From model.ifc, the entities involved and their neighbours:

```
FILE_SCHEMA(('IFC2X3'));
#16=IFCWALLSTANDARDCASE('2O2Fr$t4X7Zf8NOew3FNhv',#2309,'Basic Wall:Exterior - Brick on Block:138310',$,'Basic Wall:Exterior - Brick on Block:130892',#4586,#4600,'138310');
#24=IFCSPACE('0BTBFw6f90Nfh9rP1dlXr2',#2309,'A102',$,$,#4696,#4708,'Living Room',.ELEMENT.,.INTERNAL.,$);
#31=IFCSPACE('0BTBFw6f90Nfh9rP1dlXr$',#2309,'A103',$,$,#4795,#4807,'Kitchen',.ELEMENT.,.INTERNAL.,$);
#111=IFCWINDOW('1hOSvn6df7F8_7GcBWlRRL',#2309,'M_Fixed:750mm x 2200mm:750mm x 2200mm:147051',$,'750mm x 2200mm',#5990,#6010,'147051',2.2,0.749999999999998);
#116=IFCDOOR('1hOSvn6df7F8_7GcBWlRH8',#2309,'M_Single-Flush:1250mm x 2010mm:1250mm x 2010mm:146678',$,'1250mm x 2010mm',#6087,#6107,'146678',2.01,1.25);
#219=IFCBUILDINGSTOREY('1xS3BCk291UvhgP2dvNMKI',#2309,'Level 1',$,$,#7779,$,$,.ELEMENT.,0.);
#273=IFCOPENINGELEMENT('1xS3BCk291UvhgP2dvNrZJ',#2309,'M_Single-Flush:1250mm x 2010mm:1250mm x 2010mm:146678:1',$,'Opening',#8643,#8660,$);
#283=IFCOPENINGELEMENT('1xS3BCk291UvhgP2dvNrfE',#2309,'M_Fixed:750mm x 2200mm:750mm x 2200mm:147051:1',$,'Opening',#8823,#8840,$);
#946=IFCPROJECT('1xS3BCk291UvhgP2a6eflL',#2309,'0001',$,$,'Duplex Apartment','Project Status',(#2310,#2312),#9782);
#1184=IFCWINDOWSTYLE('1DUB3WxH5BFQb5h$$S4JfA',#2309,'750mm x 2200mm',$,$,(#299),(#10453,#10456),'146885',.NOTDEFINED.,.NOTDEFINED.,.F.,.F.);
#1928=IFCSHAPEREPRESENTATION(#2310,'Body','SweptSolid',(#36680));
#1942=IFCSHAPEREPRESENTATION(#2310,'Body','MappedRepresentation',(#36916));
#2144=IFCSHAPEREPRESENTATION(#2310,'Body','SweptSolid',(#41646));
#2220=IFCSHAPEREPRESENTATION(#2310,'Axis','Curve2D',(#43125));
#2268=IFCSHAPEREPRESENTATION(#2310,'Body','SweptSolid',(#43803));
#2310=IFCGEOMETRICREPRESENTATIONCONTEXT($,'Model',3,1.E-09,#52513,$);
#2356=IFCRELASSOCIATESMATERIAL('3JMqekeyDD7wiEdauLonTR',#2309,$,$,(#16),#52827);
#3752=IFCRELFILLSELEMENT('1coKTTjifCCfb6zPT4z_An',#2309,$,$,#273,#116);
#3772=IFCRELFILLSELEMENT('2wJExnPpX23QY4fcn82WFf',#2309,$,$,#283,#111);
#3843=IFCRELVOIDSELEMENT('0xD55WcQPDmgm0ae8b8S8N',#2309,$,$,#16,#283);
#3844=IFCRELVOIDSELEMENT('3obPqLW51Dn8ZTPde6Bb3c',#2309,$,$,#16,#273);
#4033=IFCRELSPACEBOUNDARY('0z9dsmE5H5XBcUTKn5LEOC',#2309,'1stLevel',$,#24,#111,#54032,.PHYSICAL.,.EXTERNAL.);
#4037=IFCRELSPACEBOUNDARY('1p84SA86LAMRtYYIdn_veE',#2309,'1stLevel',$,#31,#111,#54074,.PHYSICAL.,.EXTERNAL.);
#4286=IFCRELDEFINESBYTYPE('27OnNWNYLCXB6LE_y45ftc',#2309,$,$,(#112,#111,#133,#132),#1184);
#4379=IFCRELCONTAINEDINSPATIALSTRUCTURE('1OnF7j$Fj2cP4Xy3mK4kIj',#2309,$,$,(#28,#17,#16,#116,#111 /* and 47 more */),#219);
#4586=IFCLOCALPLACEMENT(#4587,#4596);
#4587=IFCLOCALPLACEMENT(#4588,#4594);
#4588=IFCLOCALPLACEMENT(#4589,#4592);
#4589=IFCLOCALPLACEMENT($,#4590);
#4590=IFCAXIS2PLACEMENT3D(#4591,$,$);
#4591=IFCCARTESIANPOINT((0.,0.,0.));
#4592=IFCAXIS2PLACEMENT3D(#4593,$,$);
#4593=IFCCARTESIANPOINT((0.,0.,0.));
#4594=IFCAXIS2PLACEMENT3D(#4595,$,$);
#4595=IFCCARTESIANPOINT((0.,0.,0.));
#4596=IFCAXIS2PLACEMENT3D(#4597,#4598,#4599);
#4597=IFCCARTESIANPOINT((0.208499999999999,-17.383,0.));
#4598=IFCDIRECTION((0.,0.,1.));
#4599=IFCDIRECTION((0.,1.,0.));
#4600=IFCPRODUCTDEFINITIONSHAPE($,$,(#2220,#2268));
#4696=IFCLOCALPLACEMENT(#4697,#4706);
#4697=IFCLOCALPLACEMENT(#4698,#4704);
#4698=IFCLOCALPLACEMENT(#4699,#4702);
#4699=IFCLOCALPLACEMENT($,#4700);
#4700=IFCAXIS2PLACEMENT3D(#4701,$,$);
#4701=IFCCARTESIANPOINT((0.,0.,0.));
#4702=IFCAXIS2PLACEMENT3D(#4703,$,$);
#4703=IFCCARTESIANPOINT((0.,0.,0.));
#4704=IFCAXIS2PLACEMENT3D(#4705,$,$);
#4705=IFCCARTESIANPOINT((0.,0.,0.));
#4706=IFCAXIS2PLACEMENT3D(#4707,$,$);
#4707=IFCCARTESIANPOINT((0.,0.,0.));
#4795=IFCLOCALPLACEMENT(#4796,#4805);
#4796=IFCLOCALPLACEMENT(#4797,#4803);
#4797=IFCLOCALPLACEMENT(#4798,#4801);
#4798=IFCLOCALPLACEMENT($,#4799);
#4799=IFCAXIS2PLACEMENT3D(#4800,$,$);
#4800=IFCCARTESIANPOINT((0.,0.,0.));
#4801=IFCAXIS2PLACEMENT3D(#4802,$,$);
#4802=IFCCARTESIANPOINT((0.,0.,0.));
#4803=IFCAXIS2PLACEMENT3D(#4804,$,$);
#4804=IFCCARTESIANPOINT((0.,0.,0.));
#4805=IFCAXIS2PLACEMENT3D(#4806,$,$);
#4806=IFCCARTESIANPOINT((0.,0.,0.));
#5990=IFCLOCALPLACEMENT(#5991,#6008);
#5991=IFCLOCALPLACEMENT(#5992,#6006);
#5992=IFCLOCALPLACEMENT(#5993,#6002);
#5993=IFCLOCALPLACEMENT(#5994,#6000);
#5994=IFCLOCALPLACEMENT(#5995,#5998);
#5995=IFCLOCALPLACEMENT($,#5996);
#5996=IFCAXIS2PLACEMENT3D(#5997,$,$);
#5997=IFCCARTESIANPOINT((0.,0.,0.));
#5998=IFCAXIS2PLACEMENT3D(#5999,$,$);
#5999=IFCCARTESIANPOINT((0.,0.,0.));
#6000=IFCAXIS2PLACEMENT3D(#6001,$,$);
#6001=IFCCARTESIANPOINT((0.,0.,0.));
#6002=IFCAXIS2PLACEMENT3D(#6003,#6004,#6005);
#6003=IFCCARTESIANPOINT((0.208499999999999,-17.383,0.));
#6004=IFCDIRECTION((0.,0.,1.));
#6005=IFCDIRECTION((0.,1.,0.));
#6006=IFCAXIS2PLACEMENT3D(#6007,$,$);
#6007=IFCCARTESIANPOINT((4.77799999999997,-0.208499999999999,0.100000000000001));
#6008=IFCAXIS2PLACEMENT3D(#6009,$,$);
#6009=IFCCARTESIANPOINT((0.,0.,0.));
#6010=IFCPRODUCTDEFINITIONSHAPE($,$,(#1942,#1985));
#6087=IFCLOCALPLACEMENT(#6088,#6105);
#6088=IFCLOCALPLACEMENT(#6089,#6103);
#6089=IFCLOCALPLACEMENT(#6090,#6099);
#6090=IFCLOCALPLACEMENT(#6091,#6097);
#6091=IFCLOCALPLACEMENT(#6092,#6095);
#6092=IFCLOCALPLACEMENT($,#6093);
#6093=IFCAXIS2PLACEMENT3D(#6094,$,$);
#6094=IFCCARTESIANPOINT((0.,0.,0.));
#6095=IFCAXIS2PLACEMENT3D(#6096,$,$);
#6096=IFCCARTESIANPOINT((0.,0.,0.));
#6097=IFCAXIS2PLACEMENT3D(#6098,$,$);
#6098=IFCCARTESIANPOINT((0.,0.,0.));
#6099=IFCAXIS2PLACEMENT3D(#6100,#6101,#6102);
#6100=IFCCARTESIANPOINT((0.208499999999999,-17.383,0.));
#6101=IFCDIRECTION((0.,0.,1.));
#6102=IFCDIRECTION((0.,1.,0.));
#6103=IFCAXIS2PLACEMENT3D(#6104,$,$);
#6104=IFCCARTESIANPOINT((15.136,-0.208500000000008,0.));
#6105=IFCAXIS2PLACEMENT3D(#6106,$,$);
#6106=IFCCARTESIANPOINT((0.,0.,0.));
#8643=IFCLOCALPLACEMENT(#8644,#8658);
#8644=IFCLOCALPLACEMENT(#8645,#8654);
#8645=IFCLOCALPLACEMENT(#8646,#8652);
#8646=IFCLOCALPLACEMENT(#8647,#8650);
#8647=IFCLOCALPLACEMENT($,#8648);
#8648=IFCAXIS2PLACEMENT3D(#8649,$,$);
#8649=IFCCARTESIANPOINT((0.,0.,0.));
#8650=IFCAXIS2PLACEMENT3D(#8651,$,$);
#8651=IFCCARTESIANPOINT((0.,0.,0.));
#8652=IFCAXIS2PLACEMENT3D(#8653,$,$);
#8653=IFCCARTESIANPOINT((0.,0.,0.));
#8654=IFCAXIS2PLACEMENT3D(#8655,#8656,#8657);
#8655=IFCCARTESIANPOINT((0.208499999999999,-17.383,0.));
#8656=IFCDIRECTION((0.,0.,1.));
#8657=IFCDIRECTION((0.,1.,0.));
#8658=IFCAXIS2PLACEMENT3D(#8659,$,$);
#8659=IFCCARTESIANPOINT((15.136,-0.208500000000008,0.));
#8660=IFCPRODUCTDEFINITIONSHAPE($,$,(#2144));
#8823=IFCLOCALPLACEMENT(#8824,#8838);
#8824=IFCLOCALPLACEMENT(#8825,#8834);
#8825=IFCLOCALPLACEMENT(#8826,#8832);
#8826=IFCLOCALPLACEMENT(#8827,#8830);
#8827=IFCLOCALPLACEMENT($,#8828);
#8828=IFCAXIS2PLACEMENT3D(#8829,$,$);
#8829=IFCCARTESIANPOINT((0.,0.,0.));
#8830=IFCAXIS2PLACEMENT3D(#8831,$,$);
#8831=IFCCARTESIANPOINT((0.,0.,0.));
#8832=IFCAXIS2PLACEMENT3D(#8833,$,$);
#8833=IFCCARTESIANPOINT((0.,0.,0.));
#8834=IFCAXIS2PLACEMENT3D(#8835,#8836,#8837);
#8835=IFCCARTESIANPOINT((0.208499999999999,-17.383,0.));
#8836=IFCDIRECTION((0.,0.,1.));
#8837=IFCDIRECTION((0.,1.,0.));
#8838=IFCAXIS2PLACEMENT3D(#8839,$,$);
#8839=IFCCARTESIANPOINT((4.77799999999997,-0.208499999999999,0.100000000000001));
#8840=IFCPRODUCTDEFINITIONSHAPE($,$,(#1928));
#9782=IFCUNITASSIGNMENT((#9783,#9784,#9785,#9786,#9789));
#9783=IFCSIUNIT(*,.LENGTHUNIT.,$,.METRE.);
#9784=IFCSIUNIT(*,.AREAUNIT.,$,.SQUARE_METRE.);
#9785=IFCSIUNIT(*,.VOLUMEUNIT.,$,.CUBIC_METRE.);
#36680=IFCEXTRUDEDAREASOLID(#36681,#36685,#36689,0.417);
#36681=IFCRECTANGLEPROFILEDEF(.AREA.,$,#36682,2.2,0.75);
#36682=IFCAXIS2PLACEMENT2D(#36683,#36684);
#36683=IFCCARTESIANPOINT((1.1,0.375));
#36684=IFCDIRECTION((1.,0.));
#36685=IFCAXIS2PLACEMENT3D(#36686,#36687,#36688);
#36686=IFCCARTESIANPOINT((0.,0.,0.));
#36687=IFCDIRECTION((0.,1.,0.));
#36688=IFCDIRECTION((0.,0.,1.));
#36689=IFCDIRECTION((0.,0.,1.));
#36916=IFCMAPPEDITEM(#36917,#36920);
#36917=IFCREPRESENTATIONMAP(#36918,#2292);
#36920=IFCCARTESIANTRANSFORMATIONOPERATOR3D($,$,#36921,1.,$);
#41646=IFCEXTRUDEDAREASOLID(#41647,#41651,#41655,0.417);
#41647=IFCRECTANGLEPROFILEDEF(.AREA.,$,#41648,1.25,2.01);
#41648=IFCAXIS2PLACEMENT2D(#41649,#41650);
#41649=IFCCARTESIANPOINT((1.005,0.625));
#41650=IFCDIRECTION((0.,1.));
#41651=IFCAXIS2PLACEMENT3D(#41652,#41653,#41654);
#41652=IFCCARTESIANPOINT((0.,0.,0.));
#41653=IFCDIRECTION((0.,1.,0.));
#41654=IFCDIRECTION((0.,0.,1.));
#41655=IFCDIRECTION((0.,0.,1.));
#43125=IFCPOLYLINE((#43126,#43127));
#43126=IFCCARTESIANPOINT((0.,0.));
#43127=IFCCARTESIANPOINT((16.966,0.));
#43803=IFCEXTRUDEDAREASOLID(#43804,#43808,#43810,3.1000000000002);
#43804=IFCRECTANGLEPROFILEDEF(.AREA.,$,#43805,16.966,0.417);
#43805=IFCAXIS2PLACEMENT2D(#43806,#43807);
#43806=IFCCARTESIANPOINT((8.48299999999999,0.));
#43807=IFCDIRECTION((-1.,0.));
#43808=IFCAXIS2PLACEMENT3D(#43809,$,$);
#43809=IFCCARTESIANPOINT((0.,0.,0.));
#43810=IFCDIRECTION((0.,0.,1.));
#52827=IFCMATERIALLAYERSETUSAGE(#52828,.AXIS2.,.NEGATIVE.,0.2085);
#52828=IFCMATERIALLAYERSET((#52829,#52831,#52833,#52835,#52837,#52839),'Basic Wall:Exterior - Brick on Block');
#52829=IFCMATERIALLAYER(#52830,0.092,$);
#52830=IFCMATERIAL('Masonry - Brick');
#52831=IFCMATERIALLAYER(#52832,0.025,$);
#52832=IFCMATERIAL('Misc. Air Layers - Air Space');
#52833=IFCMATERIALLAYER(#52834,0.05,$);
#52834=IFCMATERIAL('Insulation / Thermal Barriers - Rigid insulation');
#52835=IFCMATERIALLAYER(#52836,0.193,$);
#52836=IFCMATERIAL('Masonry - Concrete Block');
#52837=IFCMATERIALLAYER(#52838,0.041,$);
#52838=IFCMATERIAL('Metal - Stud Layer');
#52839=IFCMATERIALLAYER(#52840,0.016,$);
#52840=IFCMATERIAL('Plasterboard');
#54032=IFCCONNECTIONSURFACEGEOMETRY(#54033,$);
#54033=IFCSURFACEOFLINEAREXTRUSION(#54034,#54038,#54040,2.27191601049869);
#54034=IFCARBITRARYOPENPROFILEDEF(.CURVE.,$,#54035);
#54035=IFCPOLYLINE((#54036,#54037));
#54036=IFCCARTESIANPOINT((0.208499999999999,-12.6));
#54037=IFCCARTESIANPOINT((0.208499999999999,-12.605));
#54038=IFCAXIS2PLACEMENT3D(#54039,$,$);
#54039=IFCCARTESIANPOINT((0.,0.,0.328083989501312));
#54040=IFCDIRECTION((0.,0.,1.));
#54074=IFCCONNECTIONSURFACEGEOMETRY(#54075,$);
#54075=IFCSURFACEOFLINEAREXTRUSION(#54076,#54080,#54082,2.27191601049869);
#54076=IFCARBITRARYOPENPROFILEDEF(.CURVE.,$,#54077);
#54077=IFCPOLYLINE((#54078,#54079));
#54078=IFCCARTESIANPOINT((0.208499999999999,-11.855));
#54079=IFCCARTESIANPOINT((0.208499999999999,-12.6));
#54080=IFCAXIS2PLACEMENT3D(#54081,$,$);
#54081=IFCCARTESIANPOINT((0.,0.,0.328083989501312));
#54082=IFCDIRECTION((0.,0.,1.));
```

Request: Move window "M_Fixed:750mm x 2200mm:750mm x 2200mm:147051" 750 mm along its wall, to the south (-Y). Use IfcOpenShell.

```python
import numpy as np
import ifcopenshell
import ifcopenshell.api.geometry
import ifcopenshell.util.placement

model = ifcopenshell.open("model.ifc")

window = model.by_guid("1hOSvn6df7F8_7GcBWlRRL")
opening = window.FillsVoids[0].RelatingOpeningElement
wall = opening.VoidsElements[0].RelatingBuildingElement

wall_matrix = ifcopenshell.util.placement.get_local_placement(wall.ObjectPlacement)
shift = wall_matrix[:3, 0] * -0.75
before = ifcopenshell.util.placement.get_local_placement(window.ObjectPlacement)[:3, 3].copy()

# The window is not placed relative to its opening, so move both.
for product in (opening, window):
    matrix = ifcopenshell.util.placement.get_local_placement(product.ObjectPlacement)
    matrix[:3, 3] += shift
    ifcopenshell.api.geometry.edit_object_placement(model, product=product, matrix=matrix, is_si=False)

# Space boundary surfaces are stored in each space's coordinates; move them too.
for rel in window.ProvidesBoundaries:
    if not rel.ConnectionGeometry:
        continue
    surface = rel.ConnectionGeometry.SurfaceOnRelatingElement
    space_matrix = ifcopenshell.util.placement.get_local_placement(rel.RelatingSpace.ObjectPlacement)
    point = np.array(surface.Position.Location.Coordinates) + space_matrix[:3, :3].T @ shift
    surface.Position = model.createIfcAxis2Placement3D(
        model.createIfcCartesianPoint(point.tolist()), surface.Position.Axis, surface.Position.RefDirection
    )

after = ifcopenshell.util.placement.get_local_placement(window.ObjectPlacement)[:3, 3]
print("window moved by", (after - before).round(3) + 0.0)

model.write("model_rev.ifc")
```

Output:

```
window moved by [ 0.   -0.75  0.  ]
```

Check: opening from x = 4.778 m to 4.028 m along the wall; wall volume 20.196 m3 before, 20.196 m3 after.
